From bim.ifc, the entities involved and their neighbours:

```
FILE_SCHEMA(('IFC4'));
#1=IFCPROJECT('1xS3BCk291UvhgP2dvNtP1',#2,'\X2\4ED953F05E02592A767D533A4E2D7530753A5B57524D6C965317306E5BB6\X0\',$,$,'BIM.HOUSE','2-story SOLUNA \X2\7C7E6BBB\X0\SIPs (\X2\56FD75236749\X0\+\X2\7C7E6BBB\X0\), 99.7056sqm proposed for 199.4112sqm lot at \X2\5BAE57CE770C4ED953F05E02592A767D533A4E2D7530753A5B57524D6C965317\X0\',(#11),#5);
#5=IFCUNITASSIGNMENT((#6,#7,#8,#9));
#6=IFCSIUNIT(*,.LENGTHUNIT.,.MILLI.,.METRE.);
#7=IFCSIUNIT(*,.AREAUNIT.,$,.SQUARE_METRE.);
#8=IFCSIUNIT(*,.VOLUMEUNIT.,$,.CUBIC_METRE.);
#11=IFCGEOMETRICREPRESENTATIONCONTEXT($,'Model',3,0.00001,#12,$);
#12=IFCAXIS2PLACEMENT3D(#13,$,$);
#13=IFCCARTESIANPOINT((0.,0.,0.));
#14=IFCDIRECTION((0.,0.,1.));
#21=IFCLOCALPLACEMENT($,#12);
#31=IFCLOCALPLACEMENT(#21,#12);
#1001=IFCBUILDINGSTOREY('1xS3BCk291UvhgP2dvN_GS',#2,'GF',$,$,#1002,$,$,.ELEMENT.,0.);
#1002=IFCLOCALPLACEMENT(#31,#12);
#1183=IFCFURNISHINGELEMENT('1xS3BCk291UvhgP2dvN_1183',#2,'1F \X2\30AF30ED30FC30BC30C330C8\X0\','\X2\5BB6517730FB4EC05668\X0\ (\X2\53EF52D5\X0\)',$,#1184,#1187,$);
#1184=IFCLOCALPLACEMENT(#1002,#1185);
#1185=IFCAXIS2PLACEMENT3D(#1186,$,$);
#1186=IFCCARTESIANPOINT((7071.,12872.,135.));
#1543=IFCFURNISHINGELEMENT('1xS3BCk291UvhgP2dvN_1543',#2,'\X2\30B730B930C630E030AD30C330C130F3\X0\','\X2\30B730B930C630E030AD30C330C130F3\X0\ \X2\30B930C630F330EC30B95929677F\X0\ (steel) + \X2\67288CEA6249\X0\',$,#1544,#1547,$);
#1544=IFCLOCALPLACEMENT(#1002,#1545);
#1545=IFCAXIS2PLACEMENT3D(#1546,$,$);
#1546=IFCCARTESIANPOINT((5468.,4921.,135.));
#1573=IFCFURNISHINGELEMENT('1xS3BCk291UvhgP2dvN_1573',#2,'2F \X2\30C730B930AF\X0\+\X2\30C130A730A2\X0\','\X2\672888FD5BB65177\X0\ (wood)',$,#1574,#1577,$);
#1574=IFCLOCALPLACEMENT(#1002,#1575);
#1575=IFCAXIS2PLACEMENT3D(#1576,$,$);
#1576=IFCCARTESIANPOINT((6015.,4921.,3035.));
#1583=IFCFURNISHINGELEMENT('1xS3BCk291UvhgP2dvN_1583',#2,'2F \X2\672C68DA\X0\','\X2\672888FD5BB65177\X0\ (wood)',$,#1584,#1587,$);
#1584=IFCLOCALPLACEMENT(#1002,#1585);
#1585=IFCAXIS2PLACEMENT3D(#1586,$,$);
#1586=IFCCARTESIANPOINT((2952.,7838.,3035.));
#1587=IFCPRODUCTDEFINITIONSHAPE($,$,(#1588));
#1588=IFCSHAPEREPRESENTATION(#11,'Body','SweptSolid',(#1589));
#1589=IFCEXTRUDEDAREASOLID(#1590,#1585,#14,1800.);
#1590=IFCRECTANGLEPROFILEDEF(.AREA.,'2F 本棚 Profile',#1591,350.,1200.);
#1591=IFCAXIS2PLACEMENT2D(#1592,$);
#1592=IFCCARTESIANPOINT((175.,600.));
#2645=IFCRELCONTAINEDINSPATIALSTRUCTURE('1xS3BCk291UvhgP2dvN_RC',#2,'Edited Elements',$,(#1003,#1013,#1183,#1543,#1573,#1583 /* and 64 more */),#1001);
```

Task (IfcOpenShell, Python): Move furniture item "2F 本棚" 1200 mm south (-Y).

```python
import ifcopenshell
import ifcopenshell.api.geometry
import ifcopenshell.util.placement

model = ifcopenshell.open("bim.ifc")

item = model.by_guid("1xS3BCk291UvhgP2dvN_1583")
matrix = ifcopenshell.util.placement.get_local_placement(item.ObjectPlacement)
matrix[1, 3] -= 1200.0
ifcopenshell.api.geometry.edit_object_placement(model, product=item, matrix=matrix, is_si=False)

print(ifcopenshell.util.placement.get_local_placement(item.ObjectPlacement).round(3) + 0.0)

model.write("bim_v2.ifc")
```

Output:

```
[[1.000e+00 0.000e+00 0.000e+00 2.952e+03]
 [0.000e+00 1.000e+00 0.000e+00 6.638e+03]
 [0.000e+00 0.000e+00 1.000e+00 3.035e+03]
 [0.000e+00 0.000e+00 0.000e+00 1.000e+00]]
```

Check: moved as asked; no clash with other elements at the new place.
